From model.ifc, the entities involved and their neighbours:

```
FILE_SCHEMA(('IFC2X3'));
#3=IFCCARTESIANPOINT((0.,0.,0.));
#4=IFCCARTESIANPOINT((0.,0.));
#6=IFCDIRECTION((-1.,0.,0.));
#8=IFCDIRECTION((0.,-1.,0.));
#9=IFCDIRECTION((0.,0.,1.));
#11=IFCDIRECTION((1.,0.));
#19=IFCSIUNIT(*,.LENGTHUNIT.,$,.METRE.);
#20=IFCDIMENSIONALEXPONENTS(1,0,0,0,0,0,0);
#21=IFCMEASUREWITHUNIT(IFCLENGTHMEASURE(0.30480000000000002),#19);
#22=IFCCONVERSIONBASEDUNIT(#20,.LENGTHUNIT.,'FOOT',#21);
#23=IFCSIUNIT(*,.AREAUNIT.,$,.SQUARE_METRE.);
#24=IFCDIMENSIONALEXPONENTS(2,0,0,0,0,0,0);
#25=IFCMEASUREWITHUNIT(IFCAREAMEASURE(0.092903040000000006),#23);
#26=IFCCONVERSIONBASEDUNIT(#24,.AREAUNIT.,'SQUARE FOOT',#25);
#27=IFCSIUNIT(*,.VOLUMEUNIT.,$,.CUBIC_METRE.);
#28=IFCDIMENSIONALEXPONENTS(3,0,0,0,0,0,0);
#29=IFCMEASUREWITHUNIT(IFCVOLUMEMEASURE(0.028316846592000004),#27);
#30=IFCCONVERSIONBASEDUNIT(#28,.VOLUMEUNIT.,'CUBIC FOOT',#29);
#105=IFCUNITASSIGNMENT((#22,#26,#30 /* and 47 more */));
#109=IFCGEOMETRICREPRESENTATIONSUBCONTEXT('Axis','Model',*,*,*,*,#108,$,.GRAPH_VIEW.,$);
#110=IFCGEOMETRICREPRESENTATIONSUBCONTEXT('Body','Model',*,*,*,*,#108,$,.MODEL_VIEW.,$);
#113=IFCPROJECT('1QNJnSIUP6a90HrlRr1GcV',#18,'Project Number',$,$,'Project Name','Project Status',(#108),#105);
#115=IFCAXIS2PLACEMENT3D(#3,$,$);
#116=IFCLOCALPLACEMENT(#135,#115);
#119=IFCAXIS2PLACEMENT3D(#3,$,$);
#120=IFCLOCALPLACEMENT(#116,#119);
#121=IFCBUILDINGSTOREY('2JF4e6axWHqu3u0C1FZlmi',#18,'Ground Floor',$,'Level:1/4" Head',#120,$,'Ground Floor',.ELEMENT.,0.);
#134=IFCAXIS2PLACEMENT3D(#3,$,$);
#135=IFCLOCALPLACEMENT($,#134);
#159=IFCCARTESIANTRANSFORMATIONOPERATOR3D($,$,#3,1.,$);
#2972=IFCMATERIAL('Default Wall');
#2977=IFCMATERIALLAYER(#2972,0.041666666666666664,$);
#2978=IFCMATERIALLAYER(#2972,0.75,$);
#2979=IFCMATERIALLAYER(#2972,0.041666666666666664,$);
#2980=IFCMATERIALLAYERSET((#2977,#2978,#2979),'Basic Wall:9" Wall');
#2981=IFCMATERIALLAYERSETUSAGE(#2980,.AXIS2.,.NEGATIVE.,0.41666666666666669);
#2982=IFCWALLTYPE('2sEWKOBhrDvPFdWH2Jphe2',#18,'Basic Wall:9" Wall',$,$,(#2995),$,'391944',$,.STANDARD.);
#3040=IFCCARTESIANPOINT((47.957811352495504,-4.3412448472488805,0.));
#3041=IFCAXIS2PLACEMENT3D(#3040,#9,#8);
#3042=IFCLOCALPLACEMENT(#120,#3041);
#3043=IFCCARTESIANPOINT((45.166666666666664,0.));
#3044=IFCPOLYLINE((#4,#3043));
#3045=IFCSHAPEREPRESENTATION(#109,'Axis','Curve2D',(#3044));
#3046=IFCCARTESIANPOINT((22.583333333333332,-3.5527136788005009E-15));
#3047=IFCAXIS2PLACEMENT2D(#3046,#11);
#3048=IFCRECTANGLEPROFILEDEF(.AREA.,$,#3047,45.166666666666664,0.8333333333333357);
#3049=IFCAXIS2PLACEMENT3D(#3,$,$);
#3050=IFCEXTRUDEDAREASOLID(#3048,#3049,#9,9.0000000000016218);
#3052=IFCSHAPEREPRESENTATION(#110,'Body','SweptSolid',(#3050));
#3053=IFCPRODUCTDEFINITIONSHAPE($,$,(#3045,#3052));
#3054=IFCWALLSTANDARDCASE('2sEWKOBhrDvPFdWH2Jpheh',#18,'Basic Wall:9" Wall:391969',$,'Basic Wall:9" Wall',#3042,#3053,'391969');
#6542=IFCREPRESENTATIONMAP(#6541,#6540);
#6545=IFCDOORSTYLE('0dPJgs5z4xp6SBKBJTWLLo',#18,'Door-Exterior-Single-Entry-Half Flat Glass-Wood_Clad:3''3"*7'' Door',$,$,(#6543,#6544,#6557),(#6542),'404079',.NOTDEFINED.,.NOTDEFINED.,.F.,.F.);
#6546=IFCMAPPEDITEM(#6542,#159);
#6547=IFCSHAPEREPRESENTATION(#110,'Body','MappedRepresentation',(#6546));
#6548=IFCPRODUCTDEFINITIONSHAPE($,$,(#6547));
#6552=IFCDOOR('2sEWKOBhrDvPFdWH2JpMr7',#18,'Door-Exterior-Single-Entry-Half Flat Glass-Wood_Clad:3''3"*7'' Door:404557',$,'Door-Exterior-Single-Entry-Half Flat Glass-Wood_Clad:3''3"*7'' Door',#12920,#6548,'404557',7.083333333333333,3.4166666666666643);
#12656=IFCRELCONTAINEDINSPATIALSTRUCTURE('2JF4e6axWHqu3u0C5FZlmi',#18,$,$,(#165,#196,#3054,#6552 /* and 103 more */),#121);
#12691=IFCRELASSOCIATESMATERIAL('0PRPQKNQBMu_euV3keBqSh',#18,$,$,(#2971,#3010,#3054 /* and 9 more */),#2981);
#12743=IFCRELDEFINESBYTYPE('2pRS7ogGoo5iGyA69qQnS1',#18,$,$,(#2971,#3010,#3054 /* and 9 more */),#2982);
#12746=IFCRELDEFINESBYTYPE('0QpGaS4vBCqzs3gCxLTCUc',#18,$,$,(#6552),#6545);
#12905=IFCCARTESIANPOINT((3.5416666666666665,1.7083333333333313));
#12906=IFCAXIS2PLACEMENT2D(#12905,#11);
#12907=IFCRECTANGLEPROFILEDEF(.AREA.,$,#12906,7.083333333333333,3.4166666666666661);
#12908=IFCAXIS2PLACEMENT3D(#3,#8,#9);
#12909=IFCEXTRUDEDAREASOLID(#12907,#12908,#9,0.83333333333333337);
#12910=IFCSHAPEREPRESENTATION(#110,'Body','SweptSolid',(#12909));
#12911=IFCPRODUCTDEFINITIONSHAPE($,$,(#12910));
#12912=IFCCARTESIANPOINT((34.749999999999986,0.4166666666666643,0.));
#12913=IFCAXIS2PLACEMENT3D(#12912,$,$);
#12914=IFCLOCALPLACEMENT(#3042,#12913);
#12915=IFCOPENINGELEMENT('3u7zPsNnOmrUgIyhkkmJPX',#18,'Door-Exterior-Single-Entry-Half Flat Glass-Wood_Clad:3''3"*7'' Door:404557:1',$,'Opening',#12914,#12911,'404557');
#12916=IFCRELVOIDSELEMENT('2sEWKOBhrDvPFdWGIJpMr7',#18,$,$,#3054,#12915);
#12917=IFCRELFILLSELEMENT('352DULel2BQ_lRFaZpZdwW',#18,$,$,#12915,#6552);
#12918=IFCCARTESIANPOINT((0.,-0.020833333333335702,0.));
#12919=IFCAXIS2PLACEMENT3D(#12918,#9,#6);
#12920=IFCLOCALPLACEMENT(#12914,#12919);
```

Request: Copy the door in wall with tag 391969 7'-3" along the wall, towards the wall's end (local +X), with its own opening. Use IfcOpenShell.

```python
import ifcopenshell
import ifcopenshell.api.feature
import ifcopenshell.api.geometry
import ifcopenshell.api.root
import ifcopenshell.geom
import ifcopenshell.util.element
import ifcopenshell.util.placement
import ifcopenshell.util.shape
import ifcopenshell.util.unit

model = ifcopenshell.open("model.ifc")
unit_scale = ifcopenshell.util.unit.calculate_unit_scale(model)
settings = ifcopenshell.geom.settings()


def volume(element):
    """Net volume in cubic metres, openings subtracted."""
    shape = ifcopenshell.geom.create_shape(settings, element)
    return ifcopenshell.util.shape.get_volume(shape.geometry)


def reuse_history(source, copy):
    """copy_class also copies each property set's owner history, people and application; keep the originals."""
    for rel in copy.IsDefinedBy:
        if rel.is_a("IfcRelDefinesByProperties") and (history := rel.RelatingPropertyDefinition.OwnerHistory):
            rel.RelatingPropertyDefinition.OwnerHistory = source.OwnerHistory
            ifcopenshell.util.element.remove_deep2(model, history)


door = model.by_guid("2sEWKOBhrDvPFdWH2JpMr7")
opening = door.FillsVoids[0].RelatingOpeningElement
wall = opening.VoidsElements[0].RelatingBuildingElement
before = volume(wall)
shift = ifcopenshell.util.placement.get_local_placement(wall.ObjectPlacement)[:3, 0] * 87 * 0.0254 / unit_scale

# copy_class copies the void relationship, type, container and properties, but no geometry.
new_opening = ifcopenshell.api.root.copy_class(model, product=opening)
new_opening.Representation = ifcopenshell.util.element.copy_deep(
    model, opening.Representation, exclude=["IfcGeometricRepresentationContext", "IfcRepresentationMap"]
)
new_opening.Name = 'Door-Exterior-Single-Entry-Half Flat Glass-Wood_Clad:3\'3"*7\' Door'
new_opening.Tag = None
new_door = ifcopenshell.api.root.copy_class(model, product=door)
new_door.Representation = ifcopenshell.util.element.copy_deep(
    model, door.Representation, exclude=["IfcGeometricRepresentationContext", "IfcRepresentationMap"]
)
new_door.Name = 'Door-Exterior-Single-Entry-Half Flat Glass-Wood_Clad:3\'3"*7\' Door'
new_door.Tag = None
reuse_history(door, new_door)
fills = ifcopenshell.api.feature.add_filling(model, opening=new_opening, element=new_door)
fills.OwnerHistory = new_door.OwnerHistory  # required in IFC2X3

for old, new in ((opening, new_opening), (door, new_door)):
    matrix = ifcopenshell.util.placement.get_local_placement(old.ObjectPlacement)
    matrix[:3, 3] += shift
    ifcopenshell.api.geometry.edit_object_placement(model, product=new, matrix=matrix, is_si=False)

after = volume(wall)

print(f"wall volume {before:.3f} -> {after:.3f} m3")

model.write("model_updated.ifc")
```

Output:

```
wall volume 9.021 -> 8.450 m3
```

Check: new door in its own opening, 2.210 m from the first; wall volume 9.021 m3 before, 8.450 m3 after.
